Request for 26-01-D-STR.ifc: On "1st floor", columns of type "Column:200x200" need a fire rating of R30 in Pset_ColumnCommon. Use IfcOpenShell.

First a look at what the model holds.

```python
import ifcopenshell
import ifcopenshell.util.element

model = ifcopenshell.open("26-01-D-STR.ifc")
print(model.schema)
storey = next(s for s in model.by_type("IfcBuildingStorey") if s.Name == "1st floor")
columns = [e for e in ifcopenshell.util.element.get_decomposition(storey) if e.is_a("IfcColumn")]
seen = {}
for e in columns:
    element_type = ifcopenshell.util.element.get_type(e)
    key = (element_type.Name if element_type != e and element_type else None, ifcopenshell.util.element.get_pset(e, "Pset_ColumnCommon", "FireRating"))
    seen[key] = seen.get(key, 0) + 1
for (name, value), count in sorted(seen.items(), key=str):
    print(count, "x", name, "|", value)
```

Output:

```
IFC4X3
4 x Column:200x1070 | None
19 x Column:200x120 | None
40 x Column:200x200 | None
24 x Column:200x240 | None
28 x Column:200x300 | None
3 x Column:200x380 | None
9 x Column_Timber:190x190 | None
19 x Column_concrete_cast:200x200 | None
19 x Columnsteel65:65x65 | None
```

```python
import ifcopenshell
import ifcopenshell.api.pset
import ifcopenshell.util.element

model = ifcopenshell.open("26-01-D-STR.ifc")

storey = next(s for s in model.by_type("IfcBuildingStorey") if s.Name == "1st floor")
columns = [e for e in ifcopenshell.util.element.get_decomposition(storey) if e.is_a("IfcColumn")]

count = 0
for e in columns:
    element_type = ifcopenshell.util.element.get_type(e)
    if element_type in (None, e) or element_type.Name != "Column:200x200":
        continue
    # add_pset returns the element's existing set when there is one.
    pset = ifcopenshell.api.pset.add_pset(model, product=e, name="Pset_ColumnCommon")
    ifcopenshell.api.pset.edit_pset(model, pset=pset, properties={"FireRating": "R30"})
    count += 1

print(count, "columns updated")

model.write("26-01-D-STR-out.ifc")
```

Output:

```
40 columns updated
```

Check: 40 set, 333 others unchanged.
